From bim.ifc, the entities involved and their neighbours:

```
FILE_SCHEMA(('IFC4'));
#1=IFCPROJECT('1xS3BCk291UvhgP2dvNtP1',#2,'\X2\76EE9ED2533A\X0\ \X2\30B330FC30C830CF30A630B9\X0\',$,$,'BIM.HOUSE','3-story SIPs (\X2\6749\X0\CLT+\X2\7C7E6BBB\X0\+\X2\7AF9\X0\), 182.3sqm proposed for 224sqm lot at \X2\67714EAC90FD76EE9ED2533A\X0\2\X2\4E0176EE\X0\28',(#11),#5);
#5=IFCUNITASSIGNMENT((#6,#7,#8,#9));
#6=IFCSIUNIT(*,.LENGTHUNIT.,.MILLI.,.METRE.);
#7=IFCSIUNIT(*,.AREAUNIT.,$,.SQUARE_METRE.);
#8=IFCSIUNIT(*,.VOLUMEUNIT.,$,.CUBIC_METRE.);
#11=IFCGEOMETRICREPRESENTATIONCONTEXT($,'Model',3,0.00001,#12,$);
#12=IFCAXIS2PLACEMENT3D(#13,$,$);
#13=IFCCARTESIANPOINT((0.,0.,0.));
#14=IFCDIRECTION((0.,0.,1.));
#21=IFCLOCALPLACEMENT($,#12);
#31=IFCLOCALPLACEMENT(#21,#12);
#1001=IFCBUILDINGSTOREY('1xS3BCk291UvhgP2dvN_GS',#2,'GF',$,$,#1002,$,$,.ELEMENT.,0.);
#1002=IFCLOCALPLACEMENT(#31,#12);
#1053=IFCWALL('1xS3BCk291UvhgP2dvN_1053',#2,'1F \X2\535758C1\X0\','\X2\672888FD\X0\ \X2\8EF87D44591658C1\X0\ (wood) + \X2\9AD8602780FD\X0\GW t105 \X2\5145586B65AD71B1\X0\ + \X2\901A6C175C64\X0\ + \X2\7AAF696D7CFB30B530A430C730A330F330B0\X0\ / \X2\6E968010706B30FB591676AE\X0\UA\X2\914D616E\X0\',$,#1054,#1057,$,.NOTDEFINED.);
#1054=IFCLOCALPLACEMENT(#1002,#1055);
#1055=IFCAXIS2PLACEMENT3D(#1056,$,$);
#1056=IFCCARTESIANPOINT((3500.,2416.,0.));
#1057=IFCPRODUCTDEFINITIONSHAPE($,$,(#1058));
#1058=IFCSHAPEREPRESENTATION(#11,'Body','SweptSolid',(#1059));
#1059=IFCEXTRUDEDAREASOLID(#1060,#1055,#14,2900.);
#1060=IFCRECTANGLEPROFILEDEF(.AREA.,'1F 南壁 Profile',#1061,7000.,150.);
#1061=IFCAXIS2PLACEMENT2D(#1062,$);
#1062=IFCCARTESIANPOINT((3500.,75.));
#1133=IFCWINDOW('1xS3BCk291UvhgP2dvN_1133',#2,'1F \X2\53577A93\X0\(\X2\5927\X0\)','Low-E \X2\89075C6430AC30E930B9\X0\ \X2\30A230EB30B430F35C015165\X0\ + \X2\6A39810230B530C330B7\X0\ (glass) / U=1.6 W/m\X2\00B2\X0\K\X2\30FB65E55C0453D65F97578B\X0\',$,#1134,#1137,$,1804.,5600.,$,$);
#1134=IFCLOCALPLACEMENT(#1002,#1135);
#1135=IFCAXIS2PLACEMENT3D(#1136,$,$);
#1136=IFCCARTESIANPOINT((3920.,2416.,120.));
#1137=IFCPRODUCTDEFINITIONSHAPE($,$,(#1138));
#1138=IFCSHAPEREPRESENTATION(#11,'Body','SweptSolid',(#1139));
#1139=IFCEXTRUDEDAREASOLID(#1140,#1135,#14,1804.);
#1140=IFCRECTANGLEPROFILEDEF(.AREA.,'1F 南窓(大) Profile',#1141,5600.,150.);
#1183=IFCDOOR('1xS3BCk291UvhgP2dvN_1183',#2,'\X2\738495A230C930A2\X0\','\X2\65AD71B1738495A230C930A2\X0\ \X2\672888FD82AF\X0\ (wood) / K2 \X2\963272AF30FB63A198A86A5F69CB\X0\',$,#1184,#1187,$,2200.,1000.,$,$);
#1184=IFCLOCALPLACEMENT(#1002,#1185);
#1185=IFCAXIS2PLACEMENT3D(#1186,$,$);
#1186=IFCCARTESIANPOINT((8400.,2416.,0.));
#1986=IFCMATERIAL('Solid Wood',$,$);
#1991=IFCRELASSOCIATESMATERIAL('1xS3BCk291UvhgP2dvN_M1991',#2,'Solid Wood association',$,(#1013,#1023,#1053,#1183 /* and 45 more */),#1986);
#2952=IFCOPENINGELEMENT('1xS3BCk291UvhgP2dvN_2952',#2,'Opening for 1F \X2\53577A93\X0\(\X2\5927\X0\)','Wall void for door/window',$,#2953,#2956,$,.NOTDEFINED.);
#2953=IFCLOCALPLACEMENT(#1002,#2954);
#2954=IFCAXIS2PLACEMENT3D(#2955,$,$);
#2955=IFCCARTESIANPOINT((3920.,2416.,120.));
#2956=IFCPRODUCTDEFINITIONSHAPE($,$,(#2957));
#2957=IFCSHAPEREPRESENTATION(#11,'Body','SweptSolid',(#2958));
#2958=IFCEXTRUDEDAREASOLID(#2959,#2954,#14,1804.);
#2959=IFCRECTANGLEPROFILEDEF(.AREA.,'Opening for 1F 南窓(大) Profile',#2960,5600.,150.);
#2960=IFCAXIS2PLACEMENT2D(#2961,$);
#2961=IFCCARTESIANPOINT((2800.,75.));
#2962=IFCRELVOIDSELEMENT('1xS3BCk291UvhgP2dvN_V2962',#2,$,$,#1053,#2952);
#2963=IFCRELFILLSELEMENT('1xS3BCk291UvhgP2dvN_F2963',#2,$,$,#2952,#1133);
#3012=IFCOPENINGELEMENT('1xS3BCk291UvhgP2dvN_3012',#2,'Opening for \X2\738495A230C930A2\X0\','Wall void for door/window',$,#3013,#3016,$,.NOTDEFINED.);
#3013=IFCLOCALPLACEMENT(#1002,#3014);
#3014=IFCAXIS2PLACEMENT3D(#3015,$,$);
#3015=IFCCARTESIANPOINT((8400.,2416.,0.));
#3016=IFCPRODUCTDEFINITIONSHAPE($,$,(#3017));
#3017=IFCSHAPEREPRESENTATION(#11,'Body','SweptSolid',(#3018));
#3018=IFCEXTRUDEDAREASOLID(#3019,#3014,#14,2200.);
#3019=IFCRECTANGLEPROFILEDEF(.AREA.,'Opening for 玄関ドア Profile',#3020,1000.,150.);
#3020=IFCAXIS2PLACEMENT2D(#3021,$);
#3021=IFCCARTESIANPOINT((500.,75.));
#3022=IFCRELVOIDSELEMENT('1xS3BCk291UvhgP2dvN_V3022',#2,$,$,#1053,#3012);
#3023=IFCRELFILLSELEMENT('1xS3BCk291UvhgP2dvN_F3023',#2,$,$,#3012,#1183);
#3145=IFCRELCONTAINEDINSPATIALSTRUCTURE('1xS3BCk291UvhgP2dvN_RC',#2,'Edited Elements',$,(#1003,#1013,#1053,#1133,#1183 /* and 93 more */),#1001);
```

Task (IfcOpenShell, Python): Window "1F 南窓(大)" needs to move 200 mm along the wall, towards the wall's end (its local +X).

```python
import ifcopenshell
import ifcopenshell.api.geometry
import ifcopenshell.util.placement
import ifcopenshell.util.unit

model = ifcopenshell.open("bim.ifc")
unit_scale = ifcopenshell.util.unit.calculate_unit_scale(model)

window = model.by_id(1133)
opening = window.FillsVoids[0].RelatingOpeningElement
wall = opening.VoidsElements[0].RelatingBuildingElement

wall_matrix = ifcopenshell.util.placement.get_local_placement(wall.ObjectPlacement)
shift = wall_matrix[:3, 0] * 0.2 / unit_scale
before = ifcopenshell.util.placement.get_local_placement(window.ObjectPlacement)[:3, 3].copy()

# The window is not placed relative to its opening, so move both.
for product in (opening, window):
    matrix = ifcopenshell.util.placement.get_local_placement(product.ObjectPlacement)
    matrix[:3, 3] += shift
    ifcopenshell.api.geometry.edit_object_placement(model, product=product, matrix=matrix, is_si=False)

after = ifcopenshell.util.placement.get_local_placement(window.ObjectPlacement)[:3, 3]
print("window moved by", (after - before).round(3) + 0.0)

model.write("bim_rev.ifc")
```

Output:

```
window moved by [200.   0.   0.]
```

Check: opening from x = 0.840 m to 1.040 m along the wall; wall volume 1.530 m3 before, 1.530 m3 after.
